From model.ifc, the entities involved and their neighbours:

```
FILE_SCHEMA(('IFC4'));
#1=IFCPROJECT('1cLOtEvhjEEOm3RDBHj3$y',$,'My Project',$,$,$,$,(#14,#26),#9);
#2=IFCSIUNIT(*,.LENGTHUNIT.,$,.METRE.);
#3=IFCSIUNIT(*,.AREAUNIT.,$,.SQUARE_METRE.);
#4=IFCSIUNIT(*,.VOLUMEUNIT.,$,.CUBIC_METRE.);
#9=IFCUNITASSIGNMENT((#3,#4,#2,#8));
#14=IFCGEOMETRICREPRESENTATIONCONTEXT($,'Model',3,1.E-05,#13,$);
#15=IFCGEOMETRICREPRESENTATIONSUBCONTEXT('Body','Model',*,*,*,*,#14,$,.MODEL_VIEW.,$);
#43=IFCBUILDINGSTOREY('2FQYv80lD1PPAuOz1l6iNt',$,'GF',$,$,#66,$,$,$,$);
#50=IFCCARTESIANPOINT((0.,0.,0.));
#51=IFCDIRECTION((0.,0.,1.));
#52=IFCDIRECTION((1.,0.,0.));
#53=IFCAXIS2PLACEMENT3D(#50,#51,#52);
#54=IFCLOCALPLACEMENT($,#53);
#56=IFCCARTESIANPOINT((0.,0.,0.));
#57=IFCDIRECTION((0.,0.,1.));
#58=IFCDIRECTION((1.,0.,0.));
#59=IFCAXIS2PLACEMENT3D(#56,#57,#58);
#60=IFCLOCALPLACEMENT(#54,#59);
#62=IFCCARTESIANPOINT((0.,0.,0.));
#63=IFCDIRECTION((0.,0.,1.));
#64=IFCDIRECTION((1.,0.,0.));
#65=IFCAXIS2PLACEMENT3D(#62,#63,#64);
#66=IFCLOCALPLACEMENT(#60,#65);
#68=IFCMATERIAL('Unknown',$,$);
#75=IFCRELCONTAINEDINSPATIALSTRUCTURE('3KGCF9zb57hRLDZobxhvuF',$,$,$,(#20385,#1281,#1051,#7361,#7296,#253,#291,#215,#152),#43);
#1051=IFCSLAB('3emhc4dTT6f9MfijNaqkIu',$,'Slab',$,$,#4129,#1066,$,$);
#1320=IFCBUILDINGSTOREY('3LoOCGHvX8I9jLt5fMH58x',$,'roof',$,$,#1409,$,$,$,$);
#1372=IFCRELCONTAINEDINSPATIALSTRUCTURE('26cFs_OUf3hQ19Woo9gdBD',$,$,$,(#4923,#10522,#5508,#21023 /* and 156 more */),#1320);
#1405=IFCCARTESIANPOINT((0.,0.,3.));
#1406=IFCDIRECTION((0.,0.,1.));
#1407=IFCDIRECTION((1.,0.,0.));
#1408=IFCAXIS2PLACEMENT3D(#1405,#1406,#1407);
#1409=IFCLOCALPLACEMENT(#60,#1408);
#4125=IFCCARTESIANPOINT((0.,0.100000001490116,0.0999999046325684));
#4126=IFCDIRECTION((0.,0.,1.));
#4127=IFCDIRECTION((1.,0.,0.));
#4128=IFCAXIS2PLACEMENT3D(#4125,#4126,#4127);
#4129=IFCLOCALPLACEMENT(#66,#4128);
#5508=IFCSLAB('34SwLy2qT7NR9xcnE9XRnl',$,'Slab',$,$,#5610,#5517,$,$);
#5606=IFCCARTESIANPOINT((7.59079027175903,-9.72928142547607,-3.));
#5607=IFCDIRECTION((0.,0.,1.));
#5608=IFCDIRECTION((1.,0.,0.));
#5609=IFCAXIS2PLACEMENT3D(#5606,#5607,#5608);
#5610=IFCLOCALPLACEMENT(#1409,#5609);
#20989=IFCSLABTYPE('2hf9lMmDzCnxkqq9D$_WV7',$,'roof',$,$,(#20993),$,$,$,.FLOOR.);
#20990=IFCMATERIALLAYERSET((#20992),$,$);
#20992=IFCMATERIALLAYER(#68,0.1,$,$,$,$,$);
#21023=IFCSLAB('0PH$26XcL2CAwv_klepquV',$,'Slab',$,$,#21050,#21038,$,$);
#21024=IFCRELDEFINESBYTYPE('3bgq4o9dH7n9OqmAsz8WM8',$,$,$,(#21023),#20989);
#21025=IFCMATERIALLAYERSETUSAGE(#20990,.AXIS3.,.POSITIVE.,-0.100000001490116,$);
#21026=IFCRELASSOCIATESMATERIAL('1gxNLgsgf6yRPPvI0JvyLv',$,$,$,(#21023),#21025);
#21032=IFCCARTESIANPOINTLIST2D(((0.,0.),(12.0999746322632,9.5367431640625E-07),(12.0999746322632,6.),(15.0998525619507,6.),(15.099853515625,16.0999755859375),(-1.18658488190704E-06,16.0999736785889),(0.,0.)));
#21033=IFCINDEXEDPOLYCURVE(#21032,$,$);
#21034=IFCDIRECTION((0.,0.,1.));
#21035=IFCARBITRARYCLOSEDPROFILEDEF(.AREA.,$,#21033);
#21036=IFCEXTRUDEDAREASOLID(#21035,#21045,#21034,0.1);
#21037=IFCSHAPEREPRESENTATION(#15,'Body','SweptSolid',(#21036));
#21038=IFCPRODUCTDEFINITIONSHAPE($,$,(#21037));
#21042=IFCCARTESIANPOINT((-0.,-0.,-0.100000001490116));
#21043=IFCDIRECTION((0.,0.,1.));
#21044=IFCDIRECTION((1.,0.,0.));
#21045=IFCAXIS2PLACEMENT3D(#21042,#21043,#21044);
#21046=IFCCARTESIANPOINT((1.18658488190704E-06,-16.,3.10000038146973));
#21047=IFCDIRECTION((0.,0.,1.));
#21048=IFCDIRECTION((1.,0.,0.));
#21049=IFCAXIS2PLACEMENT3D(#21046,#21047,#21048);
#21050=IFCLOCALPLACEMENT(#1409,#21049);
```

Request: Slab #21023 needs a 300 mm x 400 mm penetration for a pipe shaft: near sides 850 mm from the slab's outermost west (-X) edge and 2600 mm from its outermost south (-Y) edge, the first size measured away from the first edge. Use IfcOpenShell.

```python
import numpy as np
import ifcopenshell
import ifcopenshell.api.feature
import ifcopenshell.api.geometry
import ifcopenshell.api.root
import ifcopenshell.geom
import ifcopenshell.util.placement
import ifcopenshell.util.representation
import ifcopenshell.util.shape
import ifcopenshell.util.unit

model = ifcopenshell.open("model.ifc")
unit_scale = ifcopenshell.util.unit.calculate_unit_scale(model)
settings = ifcopenshell.geom.settings()


def volume(element):
    """Net volume in cubic metres, openings subtracted."""
    shape = ifcopenshell.geom.create_shape(settings, element)
    return ifcopenshell.util.shape.get_volume(shape.geometry)


slab = model.by_id(21023)
before = volume(slab)

# Extent in the slab's own axes, in metres. The edges named are its -X and -Y sides.
slab_shape = ifcopenshell.geom.create_shape(settings, slab)
vertices = ifcopenshell.util.shape.get_vertices(slab_shape.geometry)
x_min, y_min, bottom = vertices.min(axis=0)
top = vertices[:, 2].max()

opening = ifcopenshell.api.root.create_entity(model, ifc_class="IfcOpeningElement", name="Pipe shaft opening", predefined_type="OPENING")
context = ifcopenshell.util.representation.get_context(model, "Model", "Body", "MODEL_VIEW")
width, depth = 0.3, 0.4
outline = [(0.0, 0.0), (width, 0.0), (width, depth), (0.0, depth), (0.0, 0.0)]
# Overshoot both faces by 50 mm so the cut is clean.
shape = ifcopenshell.api.geometry.add_slab_representation(
    model, context=context, depth=top - bottom + 0.1, polyline=outline
)
ifcopenshell.api.geometry.assign_representation(model, product=opening, representation=shape)

matrix = ifcopenshell.util.placement.get_local_placement(slab.ObjectPlacement)
matrix[:, 3] = matrix @ np.append(np.array([x_min + 0.85, y_min + 2.6, bottom - 0.05]) / unit_scale, 1.0)
ifcopenshell.api.geometry.edit_object_placement(model, product=opening, matrix=matrix, is_si=False)
ifcopenshell.api.feature.add_feature(model, feature=opening, element=slab)

after = volume(slab)

print(f"slab volume {before:.3f} -> {after:.3f} m3")

model.write("model-out.ifc")
```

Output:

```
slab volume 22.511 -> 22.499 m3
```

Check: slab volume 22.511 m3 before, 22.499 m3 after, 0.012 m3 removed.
